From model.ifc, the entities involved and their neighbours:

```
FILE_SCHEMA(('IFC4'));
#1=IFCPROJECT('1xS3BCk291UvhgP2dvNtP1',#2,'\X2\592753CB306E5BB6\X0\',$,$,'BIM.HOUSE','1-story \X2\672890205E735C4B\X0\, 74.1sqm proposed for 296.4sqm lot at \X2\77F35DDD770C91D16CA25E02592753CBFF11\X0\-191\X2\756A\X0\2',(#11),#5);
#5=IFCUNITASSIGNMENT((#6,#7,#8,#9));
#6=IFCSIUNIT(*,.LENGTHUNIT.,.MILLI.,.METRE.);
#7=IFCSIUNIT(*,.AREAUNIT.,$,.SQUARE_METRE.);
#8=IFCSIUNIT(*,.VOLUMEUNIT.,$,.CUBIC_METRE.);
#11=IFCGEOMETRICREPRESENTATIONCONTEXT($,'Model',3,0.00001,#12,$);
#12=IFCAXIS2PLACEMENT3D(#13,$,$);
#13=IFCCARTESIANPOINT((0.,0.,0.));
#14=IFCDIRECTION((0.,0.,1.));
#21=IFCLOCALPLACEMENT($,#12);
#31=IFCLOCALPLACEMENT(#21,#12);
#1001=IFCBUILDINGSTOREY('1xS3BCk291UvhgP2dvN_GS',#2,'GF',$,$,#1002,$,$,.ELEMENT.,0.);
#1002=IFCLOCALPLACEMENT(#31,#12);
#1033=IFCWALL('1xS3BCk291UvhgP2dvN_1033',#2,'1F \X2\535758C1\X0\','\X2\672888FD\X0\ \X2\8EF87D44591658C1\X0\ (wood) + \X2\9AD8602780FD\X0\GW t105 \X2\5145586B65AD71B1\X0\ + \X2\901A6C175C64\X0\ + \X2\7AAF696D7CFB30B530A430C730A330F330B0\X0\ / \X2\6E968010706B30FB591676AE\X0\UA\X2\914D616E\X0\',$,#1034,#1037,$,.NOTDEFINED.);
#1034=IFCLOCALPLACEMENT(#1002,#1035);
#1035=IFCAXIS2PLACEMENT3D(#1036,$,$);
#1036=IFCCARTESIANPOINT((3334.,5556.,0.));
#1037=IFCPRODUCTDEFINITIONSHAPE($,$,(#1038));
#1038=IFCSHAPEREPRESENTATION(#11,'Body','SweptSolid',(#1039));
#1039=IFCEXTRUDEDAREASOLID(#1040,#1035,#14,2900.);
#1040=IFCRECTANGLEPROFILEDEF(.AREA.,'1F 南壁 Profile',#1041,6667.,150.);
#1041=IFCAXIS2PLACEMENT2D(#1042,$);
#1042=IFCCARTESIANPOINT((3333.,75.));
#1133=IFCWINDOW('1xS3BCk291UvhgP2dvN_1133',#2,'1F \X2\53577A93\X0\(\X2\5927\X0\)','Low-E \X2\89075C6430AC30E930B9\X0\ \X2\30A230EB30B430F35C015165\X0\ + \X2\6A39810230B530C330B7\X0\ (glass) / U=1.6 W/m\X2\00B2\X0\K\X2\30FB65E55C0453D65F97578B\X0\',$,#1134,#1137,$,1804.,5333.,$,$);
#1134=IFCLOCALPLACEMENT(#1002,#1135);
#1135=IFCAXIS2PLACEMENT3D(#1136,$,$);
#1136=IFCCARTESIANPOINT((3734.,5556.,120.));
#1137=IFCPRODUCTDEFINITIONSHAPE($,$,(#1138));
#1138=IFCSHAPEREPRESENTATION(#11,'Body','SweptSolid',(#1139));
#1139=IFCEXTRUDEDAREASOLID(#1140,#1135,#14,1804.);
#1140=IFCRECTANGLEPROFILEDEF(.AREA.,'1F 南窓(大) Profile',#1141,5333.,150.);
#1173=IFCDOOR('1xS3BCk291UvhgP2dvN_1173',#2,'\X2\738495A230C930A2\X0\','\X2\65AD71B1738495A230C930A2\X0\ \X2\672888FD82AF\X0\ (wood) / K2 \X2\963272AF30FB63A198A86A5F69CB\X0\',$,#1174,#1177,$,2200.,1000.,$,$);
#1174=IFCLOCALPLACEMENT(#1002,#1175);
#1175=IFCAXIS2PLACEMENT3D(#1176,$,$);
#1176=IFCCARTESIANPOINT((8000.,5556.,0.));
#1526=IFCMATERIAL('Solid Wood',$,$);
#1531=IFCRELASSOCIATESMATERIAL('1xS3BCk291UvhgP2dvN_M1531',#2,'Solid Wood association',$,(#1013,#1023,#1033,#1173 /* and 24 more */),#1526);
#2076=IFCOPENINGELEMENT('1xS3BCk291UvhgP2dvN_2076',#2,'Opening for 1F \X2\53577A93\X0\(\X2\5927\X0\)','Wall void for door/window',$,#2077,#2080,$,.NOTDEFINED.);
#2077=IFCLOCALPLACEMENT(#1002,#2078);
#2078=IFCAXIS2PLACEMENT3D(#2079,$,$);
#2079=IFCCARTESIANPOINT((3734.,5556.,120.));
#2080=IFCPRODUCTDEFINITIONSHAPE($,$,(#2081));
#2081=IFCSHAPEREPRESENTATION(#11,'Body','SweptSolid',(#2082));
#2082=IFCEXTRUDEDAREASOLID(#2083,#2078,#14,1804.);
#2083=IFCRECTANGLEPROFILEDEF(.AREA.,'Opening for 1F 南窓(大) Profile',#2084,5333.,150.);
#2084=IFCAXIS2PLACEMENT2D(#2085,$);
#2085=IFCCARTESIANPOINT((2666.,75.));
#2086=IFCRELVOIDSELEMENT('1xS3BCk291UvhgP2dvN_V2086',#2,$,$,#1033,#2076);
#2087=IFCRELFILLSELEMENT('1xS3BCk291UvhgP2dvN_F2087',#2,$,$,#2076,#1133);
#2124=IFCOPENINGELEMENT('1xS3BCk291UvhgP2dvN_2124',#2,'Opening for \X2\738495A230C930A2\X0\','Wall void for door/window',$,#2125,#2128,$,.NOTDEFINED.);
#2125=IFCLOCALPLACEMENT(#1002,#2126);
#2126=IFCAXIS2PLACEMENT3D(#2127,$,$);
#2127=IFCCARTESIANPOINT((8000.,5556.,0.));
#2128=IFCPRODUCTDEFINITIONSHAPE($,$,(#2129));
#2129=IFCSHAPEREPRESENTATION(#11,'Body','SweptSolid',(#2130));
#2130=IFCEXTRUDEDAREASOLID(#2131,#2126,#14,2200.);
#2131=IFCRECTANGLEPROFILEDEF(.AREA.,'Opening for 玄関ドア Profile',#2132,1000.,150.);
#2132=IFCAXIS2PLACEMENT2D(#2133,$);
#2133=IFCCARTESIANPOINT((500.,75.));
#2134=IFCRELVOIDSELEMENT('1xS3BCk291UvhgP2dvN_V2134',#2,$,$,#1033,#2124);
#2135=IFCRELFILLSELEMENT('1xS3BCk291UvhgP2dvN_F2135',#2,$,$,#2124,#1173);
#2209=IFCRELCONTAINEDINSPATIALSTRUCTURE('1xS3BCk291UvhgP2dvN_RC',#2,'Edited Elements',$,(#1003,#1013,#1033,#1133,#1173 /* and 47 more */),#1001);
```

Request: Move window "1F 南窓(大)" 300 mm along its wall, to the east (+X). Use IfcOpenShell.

```python
import ifcopenshell
import ifcopenshell.api.geometry
import ifcopenshell.util.placement

model = ifcopenshell.open("model.ifc")

window = model.by_id(1133)
opening = window.FillsVoids[0].RelatingOpeningElement
wall = opening.VoidsElements[0].RelatingBuildingElement

wall_matrix = ifcopenshell.util.placement.get_local_placement(wall.ObjectPlacement)
shift = wall_matrix[:3, 0] * 300.0
before = ifcopenshell.util.placement.get_local_placement(window.ObjectPlacement)[:3, 3].copy()

# The window is not placed relative to its opening, so move both.
for product in (opening, window):
    matrix = ifcopenshell.util.placement.get_local_placement(product.ObjectPlacement)
    matrix[:3, 3] += shift
    ifcopenshell.api.geometry.edit_object_placement(model, product=product, matrix=matrix, is_si=False)

after = ifcopenshell.util.placement.get_local_placement(window.ObjectPlacement)[:3, 3]
print("window moved by", (after - before).round(3) + 0.0)

model.write("model-out.ifc")
```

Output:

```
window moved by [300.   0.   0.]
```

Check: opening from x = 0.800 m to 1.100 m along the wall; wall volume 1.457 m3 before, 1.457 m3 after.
